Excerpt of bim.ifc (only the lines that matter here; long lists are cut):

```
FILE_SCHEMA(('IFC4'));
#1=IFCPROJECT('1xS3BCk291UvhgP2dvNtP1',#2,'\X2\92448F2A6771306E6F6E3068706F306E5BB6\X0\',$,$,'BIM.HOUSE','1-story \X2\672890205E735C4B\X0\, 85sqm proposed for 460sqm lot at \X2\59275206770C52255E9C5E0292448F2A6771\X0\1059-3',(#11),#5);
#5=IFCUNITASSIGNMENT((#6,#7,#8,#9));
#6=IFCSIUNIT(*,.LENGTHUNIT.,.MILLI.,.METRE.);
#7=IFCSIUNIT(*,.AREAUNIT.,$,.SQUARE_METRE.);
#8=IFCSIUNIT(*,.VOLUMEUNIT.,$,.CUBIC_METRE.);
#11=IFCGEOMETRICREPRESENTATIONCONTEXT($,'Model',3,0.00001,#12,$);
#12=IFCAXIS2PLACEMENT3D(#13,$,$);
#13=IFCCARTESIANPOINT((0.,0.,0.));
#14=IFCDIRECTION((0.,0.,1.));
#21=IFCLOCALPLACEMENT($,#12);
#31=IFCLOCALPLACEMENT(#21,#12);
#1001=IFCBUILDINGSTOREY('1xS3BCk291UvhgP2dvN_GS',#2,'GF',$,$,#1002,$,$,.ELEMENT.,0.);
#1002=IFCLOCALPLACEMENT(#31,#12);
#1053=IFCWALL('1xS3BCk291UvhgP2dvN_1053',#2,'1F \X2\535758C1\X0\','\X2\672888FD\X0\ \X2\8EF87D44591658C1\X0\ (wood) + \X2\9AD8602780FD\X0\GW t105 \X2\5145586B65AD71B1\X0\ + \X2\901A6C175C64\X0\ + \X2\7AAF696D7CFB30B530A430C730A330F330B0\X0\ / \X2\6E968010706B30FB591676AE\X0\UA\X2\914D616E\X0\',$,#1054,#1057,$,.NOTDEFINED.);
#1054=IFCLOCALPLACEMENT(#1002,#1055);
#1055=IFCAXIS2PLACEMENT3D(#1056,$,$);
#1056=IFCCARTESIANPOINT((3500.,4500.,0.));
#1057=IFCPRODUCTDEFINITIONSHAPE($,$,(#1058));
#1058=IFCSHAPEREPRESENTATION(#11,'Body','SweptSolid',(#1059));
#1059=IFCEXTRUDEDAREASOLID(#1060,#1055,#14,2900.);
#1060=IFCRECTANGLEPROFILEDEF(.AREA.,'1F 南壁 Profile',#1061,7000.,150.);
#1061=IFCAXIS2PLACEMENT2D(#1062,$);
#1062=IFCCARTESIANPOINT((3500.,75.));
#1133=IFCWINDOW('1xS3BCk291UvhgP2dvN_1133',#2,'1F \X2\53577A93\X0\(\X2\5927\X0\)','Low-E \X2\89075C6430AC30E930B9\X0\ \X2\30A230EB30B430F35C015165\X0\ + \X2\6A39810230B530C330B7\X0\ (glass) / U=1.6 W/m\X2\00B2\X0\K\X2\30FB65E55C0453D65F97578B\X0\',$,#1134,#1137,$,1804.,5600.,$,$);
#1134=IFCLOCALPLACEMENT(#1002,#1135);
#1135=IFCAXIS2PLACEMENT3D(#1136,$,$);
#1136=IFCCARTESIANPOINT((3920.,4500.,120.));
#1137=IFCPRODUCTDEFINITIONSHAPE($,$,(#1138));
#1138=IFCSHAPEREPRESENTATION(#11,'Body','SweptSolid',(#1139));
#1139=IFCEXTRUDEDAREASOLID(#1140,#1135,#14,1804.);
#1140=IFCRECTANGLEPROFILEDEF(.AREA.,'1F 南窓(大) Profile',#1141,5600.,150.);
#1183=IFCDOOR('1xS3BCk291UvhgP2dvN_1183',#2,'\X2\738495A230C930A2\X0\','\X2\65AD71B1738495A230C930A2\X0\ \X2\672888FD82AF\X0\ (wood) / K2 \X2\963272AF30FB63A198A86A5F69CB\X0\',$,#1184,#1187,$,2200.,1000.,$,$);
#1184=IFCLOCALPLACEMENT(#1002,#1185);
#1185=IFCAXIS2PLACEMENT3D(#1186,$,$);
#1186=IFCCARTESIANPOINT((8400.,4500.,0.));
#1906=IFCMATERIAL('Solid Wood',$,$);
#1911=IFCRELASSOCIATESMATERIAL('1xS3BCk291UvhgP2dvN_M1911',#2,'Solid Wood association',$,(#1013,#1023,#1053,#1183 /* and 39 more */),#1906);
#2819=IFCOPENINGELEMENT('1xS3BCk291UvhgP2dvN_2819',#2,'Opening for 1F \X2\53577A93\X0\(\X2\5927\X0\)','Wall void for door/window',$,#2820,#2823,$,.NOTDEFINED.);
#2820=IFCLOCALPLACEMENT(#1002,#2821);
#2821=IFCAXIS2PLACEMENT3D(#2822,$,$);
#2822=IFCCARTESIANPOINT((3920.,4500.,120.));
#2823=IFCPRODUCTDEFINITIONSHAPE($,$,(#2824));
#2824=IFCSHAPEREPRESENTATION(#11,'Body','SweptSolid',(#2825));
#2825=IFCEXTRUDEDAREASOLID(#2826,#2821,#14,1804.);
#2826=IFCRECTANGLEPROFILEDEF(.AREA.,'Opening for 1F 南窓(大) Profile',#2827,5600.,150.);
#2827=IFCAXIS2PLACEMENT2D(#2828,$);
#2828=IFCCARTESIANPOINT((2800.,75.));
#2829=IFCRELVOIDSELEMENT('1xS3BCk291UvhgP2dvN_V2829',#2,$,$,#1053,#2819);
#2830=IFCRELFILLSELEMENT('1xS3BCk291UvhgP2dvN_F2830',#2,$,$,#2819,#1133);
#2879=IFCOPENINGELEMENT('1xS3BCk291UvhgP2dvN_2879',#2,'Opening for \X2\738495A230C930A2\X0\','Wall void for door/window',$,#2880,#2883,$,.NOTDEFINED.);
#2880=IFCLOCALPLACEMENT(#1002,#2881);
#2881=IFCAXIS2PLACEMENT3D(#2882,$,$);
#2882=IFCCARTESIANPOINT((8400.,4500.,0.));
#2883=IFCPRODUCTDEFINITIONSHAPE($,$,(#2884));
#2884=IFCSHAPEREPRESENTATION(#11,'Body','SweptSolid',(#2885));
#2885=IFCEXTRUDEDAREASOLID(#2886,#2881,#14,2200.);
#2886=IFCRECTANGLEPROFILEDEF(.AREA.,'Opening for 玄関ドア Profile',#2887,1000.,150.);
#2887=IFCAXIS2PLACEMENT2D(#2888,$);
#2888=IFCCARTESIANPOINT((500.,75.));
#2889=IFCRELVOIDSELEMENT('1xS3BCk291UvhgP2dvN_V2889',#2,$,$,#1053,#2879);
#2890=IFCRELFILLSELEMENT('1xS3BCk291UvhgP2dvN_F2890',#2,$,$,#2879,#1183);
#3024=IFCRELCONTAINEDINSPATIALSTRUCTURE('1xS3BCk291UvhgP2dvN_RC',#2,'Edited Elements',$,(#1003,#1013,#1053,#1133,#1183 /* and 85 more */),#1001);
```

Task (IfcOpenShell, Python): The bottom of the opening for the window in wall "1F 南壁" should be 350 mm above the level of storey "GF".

```python
import numpy as np
import ifcopenshell
import ifcopenshell.api.geometry
import ifcopenshell.geom
import ifcopenshell.util.element
import ifcopenshell.util.placement
import ifcopenshell.util.shape
import ifcopenshell.util.unit

model = ifcopenshell.open("bim.ifc")
unit_scale = ifcopenshell.util.unit.calculate_unit_scale(model)

window = model.by_id(1133)
opening = window.FillsVoids[0].RelatingOpeningElement
storey = ifcopenshell.util.element.get_container(window, ifc_class="IfcBuildingStorey")
level = ifcopenshell.util.placement.get_local_placement(storey.ObjectPlacement)[2, 3]

# The opening's origin need not be at the sill, so measure its lowest point.
shape = ifcopenshell.geom.create_shape(ifcopenshell.geom.settings(), opening)
bottom = ifcopenshell.util.shape.get_shape_bottom_elevation(shape, shape.geometry) / unit_scale
dz = level + 350.0 - bottom

shift = np.array([0.0, 0.0, dz])
# The window is not placed relative to its opening, so move both.
for product in (opening, window):
    matrix = ifcopenshell.util.placement.get_local_placement(product.ObjectPlacement)
    matrix[:3, 3] += shift
    ifcopenshell.api.geometry.edit_object_placement(model, product=product, matrix=matrix, is_si=False)

print(f"moved by {dz * unit_scale:+.3f} m")

model.write("bim_rev.ifc")
```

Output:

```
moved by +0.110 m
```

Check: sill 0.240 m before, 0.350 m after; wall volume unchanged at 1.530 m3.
